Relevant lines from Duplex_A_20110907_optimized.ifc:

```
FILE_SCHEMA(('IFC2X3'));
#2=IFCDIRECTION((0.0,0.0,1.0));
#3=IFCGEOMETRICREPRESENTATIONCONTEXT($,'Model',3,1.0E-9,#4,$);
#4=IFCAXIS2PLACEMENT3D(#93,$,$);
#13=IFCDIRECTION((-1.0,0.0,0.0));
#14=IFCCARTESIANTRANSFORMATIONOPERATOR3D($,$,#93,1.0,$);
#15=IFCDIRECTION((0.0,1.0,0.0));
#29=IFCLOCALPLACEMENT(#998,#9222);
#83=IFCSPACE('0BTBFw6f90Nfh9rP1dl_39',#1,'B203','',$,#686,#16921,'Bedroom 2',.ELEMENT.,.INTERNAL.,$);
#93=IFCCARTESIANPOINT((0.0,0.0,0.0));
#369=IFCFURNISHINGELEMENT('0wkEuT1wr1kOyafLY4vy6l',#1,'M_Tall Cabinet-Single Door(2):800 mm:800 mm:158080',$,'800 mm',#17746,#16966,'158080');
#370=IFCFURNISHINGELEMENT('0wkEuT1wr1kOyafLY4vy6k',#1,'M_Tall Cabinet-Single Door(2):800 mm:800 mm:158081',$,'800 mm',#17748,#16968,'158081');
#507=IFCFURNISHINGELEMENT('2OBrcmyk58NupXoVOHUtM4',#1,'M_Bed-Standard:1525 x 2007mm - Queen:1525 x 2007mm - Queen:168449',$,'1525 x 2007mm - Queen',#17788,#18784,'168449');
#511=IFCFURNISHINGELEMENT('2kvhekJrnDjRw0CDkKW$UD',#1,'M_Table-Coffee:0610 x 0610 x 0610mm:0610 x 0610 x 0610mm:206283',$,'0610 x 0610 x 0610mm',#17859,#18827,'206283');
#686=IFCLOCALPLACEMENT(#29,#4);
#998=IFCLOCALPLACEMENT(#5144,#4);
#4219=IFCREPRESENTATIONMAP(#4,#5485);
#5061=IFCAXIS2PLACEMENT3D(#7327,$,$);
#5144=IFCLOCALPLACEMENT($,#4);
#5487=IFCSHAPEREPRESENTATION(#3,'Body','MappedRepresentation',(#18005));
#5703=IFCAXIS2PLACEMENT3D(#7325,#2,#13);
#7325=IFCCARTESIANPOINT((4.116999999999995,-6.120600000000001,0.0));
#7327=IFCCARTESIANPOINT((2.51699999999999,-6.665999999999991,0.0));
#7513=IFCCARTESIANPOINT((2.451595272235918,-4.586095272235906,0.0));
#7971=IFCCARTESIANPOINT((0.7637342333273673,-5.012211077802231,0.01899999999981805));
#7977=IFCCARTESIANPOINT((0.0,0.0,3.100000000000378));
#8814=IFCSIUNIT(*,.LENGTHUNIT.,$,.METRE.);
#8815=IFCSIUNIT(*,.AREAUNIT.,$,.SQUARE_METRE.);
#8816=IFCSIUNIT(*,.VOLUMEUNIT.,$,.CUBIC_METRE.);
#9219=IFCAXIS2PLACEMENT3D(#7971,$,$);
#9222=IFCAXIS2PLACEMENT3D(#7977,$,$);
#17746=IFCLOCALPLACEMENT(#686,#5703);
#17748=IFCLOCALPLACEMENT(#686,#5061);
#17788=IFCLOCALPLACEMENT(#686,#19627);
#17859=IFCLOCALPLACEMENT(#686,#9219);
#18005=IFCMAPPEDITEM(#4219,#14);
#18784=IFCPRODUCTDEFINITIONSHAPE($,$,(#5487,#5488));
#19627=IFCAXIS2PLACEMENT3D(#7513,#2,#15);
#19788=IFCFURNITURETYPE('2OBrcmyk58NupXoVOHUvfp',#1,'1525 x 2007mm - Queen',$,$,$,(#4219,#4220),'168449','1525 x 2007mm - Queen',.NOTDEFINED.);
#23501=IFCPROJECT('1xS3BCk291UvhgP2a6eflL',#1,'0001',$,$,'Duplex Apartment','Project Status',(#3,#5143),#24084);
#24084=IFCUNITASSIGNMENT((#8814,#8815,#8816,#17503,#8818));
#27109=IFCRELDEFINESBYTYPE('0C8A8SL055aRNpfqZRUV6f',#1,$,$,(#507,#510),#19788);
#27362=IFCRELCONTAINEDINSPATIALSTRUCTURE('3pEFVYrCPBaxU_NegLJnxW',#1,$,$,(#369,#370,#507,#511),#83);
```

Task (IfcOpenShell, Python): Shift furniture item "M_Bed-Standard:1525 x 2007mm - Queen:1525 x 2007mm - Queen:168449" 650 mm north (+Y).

```python
import ifcopenshell
import ifcopenshell.api.geometry
import ifcopenshell.util.placement
import ifcopenshell.util.unit

model = ifcopenshell.open("Duplex_A_20110907_optimized.ifc")
unit_scale = ifcopenshell.util.unit.calculate_unit_scale(model)

item = model.by_id(507)
matrix = ifcopenshell.util.placement.get_local_placement(item.ObjectPlacement)
matrix[1, 3] += 0.65 / unit_scale
ifcopenshell.api.geometry.edit_object_placement(model, product=item, matrix=matrix, is_si=False)

print(ifcopenshell.util.placement.get_local_placement(item.ObjectPlacement).round(3) + 0.0)

model.write("Duplex_A_20110907_optimized_v2.ifc")
```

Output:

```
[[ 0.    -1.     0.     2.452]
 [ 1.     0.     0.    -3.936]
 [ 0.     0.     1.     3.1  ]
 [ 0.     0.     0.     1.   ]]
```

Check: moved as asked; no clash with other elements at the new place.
